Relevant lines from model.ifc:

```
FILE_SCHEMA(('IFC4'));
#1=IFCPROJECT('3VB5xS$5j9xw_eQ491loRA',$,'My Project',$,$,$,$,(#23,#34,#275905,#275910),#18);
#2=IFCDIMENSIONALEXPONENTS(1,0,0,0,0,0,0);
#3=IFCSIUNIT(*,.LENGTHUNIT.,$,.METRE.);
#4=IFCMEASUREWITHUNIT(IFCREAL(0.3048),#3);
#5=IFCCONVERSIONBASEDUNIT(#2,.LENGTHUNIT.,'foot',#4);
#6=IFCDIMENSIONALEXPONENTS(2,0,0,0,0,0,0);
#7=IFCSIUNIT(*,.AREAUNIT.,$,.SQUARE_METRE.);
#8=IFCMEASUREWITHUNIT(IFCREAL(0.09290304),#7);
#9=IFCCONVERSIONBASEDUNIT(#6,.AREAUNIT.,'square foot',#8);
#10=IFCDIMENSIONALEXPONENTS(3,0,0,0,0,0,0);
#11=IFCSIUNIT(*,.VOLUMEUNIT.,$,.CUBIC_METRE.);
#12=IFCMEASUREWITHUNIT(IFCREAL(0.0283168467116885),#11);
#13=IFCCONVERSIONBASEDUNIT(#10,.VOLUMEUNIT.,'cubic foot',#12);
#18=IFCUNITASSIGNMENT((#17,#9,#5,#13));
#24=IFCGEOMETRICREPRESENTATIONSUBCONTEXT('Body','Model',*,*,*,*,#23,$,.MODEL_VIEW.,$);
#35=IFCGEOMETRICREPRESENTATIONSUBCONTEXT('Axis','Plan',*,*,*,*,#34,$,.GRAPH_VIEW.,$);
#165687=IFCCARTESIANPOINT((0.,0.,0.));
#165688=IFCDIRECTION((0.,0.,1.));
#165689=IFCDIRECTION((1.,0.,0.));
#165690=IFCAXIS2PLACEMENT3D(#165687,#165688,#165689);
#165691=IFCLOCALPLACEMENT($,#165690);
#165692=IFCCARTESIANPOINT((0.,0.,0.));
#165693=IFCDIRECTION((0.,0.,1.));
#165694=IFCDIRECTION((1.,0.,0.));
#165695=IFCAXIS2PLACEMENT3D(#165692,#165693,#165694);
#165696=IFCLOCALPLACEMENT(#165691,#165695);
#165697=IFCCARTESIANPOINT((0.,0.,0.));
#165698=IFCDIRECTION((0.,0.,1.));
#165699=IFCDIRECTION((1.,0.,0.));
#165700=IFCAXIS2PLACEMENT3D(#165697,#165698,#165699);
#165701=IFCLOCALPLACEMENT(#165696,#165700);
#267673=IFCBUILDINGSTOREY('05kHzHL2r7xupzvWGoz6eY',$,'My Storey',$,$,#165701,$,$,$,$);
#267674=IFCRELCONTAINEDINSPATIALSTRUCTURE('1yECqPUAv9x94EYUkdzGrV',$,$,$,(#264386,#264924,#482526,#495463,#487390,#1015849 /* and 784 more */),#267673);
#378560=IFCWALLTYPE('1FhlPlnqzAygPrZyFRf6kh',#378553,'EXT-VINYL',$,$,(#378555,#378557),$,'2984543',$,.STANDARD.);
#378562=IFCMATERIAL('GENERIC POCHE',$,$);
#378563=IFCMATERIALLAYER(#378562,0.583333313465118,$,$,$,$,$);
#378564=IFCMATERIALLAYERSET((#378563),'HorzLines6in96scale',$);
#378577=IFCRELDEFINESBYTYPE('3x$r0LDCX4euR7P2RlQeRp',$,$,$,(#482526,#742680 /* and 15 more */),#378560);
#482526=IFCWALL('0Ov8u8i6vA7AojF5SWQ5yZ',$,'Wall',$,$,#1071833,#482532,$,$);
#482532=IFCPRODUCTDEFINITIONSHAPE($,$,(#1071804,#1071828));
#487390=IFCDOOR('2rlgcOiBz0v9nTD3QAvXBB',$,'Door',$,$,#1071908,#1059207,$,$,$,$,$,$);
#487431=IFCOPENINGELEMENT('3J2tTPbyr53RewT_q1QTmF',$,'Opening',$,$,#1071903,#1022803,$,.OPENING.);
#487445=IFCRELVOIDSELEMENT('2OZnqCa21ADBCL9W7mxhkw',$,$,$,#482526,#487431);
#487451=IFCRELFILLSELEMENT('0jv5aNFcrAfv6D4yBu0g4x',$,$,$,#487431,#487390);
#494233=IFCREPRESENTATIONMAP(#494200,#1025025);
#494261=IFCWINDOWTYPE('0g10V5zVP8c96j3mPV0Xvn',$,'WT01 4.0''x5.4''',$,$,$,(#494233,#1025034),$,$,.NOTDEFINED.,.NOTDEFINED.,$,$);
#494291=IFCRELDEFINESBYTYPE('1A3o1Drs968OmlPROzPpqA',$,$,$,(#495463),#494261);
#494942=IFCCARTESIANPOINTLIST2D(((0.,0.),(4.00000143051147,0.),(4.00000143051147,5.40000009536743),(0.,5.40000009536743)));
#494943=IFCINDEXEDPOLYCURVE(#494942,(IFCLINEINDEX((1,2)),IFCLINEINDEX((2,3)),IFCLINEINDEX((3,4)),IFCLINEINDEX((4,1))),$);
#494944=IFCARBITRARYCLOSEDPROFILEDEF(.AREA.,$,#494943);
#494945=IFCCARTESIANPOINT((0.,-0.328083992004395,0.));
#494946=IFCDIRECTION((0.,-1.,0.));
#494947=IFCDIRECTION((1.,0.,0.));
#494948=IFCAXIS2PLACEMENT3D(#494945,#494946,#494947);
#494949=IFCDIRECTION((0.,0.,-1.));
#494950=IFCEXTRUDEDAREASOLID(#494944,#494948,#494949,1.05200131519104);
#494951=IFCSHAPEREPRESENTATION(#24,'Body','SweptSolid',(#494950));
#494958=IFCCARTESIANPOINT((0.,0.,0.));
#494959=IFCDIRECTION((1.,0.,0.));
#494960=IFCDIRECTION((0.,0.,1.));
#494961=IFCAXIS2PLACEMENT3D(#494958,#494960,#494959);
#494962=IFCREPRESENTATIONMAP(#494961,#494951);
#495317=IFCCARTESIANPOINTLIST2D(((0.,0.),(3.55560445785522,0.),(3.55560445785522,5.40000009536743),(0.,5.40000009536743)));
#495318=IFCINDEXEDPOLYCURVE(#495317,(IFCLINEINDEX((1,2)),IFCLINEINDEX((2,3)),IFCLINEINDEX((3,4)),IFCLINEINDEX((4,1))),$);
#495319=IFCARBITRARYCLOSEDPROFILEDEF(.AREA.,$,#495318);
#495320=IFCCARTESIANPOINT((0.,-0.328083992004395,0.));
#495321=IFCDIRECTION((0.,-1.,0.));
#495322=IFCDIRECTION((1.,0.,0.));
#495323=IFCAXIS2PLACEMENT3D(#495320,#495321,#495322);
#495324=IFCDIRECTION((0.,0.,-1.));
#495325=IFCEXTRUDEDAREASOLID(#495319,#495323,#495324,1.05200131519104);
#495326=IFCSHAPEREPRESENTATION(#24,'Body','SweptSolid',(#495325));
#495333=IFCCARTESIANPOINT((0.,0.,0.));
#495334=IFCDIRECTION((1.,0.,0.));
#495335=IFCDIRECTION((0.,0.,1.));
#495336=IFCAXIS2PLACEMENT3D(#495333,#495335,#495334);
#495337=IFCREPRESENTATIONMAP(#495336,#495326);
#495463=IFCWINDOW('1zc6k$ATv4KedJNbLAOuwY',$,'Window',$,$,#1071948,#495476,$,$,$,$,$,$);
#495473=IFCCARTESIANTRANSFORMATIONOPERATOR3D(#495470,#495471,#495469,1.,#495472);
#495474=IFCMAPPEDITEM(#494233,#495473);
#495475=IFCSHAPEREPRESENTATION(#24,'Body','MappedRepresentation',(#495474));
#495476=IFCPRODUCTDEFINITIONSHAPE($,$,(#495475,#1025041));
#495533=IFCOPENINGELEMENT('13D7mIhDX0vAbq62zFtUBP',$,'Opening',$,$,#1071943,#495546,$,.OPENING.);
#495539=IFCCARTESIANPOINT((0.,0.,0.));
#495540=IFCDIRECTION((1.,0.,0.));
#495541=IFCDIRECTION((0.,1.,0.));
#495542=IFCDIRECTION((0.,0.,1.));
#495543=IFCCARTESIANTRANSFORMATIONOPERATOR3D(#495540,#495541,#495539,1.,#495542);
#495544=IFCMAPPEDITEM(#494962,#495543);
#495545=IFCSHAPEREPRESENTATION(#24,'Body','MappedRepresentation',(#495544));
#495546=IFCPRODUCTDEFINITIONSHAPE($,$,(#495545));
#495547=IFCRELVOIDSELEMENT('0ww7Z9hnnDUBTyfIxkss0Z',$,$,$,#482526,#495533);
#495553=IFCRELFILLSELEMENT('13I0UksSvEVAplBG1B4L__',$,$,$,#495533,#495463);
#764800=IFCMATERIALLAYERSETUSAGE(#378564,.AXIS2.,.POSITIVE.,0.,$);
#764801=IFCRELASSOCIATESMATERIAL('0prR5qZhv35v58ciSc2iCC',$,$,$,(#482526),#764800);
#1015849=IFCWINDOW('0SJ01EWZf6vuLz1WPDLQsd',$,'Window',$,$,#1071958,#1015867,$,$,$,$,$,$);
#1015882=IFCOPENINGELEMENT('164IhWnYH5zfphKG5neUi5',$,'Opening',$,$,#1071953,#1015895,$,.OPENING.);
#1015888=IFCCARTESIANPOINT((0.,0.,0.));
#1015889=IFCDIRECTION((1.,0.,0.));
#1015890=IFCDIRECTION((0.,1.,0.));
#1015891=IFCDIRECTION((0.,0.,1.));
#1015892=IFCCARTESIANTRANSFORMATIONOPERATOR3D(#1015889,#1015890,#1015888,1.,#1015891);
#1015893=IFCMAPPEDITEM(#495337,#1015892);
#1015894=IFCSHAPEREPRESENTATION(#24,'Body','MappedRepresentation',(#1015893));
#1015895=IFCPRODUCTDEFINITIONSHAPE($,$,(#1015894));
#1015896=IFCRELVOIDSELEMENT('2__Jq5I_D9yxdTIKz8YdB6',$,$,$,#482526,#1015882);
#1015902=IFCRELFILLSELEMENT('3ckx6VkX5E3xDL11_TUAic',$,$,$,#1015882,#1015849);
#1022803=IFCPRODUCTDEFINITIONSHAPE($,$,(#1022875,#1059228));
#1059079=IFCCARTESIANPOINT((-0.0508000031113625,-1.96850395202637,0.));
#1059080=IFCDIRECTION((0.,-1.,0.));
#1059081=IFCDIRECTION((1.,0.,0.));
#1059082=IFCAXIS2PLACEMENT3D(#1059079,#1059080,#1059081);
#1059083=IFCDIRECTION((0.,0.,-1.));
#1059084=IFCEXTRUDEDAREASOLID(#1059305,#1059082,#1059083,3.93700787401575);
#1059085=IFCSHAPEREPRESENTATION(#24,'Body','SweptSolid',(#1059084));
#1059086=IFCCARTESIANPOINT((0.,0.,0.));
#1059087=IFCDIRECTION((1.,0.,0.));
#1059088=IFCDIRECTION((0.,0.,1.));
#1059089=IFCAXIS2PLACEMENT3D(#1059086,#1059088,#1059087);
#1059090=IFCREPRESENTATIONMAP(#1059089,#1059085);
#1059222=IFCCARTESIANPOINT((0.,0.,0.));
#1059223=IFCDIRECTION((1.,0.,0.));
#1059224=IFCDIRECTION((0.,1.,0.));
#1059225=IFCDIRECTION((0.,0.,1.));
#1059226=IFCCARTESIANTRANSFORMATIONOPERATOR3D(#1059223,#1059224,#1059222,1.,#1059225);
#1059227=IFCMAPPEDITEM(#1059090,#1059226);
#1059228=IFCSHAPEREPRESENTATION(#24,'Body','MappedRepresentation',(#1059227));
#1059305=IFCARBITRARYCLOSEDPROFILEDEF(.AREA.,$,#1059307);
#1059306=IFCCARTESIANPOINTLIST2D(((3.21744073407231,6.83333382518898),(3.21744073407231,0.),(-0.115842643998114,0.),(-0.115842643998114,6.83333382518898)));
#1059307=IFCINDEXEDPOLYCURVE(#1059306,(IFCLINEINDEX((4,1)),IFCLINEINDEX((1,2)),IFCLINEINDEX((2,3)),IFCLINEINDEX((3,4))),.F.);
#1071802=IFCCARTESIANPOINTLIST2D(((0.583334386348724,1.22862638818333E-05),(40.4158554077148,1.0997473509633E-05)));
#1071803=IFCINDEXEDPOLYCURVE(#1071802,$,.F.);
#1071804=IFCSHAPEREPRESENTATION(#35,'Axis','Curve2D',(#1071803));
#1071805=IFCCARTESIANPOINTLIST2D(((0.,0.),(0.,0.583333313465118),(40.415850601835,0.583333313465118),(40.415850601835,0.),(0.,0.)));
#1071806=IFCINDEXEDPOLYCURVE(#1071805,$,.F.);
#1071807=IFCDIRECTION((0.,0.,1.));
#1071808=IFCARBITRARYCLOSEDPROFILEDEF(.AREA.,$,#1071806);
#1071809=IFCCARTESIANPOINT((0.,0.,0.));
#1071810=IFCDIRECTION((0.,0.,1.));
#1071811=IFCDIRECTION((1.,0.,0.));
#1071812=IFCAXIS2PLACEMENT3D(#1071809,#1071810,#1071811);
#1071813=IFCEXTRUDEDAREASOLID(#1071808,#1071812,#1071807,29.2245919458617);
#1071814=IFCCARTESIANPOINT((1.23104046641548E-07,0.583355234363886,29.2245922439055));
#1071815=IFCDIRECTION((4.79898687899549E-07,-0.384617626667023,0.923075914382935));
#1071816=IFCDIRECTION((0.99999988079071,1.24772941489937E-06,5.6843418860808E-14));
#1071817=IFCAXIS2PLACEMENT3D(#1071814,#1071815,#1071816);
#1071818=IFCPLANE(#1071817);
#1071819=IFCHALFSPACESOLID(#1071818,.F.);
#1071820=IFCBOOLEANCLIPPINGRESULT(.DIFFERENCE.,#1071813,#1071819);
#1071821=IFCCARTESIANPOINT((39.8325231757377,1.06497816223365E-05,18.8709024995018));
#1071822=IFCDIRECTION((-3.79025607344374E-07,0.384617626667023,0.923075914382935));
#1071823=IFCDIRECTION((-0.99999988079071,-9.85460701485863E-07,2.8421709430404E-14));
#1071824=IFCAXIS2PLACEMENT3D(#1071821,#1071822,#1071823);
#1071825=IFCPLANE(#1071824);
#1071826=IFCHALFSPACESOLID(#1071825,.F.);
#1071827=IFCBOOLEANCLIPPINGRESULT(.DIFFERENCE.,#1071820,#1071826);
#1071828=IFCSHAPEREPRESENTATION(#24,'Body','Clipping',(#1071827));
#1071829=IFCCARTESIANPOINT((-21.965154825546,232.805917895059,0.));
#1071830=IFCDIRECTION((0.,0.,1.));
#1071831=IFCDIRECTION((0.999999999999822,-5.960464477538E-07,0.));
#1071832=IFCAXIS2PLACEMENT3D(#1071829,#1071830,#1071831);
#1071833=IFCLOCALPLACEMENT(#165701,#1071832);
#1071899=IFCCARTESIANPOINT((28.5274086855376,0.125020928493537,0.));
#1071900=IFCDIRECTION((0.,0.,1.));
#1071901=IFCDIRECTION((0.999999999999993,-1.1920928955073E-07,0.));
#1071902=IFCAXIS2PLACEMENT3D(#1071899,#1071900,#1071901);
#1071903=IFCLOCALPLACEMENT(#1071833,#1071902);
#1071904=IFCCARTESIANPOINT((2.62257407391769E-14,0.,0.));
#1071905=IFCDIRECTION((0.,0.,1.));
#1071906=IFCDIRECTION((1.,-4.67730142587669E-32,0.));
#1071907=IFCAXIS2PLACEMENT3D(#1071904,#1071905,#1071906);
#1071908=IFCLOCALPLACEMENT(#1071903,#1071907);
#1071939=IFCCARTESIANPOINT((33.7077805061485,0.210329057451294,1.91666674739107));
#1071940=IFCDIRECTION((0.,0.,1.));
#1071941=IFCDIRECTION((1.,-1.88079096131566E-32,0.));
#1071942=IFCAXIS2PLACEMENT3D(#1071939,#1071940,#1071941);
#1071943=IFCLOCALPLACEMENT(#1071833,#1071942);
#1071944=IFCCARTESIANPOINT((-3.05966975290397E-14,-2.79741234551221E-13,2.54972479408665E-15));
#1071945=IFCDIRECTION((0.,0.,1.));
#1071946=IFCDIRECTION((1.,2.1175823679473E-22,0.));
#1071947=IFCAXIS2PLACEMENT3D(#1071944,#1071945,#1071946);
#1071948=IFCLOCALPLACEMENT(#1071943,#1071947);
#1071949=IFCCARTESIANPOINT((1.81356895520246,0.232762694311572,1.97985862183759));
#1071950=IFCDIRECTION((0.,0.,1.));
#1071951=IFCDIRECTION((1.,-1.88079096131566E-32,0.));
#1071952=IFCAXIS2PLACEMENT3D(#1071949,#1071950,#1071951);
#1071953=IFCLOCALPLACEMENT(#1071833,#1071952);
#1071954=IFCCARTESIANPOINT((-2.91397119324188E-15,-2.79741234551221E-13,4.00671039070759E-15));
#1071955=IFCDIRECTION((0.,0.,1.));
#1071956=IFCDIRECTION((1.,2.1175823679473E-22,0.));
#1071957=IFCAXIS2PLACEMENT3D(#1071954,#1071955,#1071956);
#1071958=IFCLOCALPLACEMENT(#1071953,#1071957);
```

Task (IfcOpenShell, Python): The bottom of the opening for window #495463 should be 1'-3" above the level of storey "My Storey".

```python
import numpy as np
import ifcopenshell
import ifcopenshell.api.geometry
import ifcopenshell.geom
import ifcopenshell.util.element
import ifcopenshell.util.placement
import ifcopenshell.util.shape
import ifcopenshell.util.unit

model = ifcopenshell.open("model.ifc")
unit_scale = ifcopenshell.util.unit.calculate_unit_scale(model)

window = model.by_guid("1zc6k$ATv4KedJNbLAOuwY")
opening = window.FillsVoids[0].RelatingOpeningElement
storey = ifcopenshell.util.element.get_container(window, ifc_class="IfcBuildingStorey")
level = ifcopenshell.util.placement.get_local_placement(storey.ObjectPlacement)[2, 3]

# The opening's origin need not be at the sill, so measure its lowest point.
shape = ifcopenshell.geom.create_shape(ifcopenshell.geom.settings(), opening)
bottom = ifcopenshell.util.shape.get_shape_bottom_elevation(shape, shape.geometry) / unit_scale
dz = level + 15 * 0.0254 / unit_scale - bottom

shift = np.array([0.0, 0.0, dz])
# The window is placed relative to its opening, so it follows when the opening moves.
matrix = ifcopenshell.util.placement.get_local_placement(opening.ObjectPlacement)
matrix[:3, 3] += shift
ifcopenshell.api.geometry.edit_object_placement(
    model, product=opening, matrix=matrix, is_si=False, should_transform_children=True
)

print(f"moved by {dz * unit_scale:+.3f} m")

model.write("model_rev.ifc")
```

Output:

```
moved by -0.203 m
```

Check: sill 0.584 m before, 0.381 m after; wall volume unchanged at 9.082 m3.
